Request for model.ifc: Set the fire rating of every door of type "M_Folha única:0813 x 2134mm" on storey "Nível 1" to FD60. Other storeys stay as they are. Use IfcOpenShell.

First a look at what the model holds.

```python
import ifcopenshell
import ifcopenshell.util.element

model = ifcopenshell.open("model.ifc")
print(model.schema)
storey = next(s for s in model.by_type("IfcBuildingStorey") if s.Name == "Nível 1")
doors = [e for e in ifcopenshell.util.element.get_decomposition(storey) if e.is_a("IfcDoor")]
seen = {}
for e in doors:
    element_type = ifcopenshell.util.element.get_type(e)
    key = (element_type.Name if element_type != e and element_type else None, ifcopenshell.util.element.get_pset(e, "Pset_DoorCommon", "FireRating"))
    seen[key] = seen.get(key, 0) + 1
for (name, value), count in sorted(seen.items(), key=str):
    print(count, "x", name, "|", value)
```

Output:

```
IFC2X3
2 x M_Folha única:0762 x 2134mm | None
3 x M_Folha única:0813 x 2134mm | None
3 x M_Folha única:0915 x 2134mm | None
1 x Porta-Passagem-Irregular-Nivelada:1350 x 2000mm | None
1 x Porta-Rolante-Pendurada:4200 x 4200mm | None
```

```python
import ifcopenshell
import ifcopenshell.api.pset
import ifcopenshell.util.element

model = ifcopenshell.open("model.ifc")

storey = next(s for s in model.by_type("IfcBuildingStorey") if s.Name == "Nível 1")
doors = [e for e in ifcopenshell.util.element.get_decomposition(storey) if e.is_a("IfcDoor")]

count = 0
for e in doors:
    element_type = ifcopenshell.util.element.get_type(e)
    if element_type in (None, e) or element_type.Name != "M_Folha única:0813 x 2134mm":
        continue
    # add_pset returns the element's existing set when there is one.
    pset = ifcopenshell.api.pset.add_pset(model, product=e, name="Pset_DoorCommon")
    ifcopenshell.api.pset.edit_pset(model, pset=pset, properties={"FireRating": "FD60"})
    count += 1

print(count, "doors updated")

model.write("model_rev.ifc")
```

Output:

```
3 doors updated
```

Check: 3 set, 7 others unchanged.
